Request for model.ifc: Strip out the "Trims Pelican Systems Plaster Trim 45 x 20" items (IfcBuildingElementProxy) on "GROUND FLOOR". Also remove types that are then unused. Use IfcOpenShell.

First a look at what the model holds.

```python
import ifcopenshell
import ifcopenshell.util.element

model = ifcopenshell.open("model.ifc")
print(model.schema)
storey = next(s for s in model.by_type("IfcBuildingStorey") if s.Name == "GROUND FLOOR")
proxies = [e for e in ifcopenshell.util.element.get_decomposition(storey) if e.is_a("IfcBuildingElementProxy")]
seen = {}
for e in proxies:
    element_type = ifcopenshell.util.element.get_type(e)
    name = element_type.Name if element_type not in (None, e) else None
    seen[name] = seen.get(name, 0) + 1
for name, count in sorted(seen.items(), key=str):
    print(count, "x", name)
```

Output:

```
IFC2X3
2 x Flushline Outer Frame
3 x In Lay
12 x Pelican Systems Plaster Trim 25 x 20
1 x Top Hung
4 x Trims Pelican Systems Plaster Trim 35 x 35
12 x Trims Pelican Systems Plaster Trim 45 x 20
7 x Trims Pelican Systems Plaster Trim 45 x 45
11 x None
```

```python
import ifcopenshell
import ifcopenshell.api.root
import ifcopenshell.util.element

model = ifcopenshell.open("model.ifc")

storey = next(s for s in model.by_type("IfcBuildingStorey") if s.Name == "GROUND FLOOR")
proxies = [e for e in ifcopenshell.util.element.get_decomposition(storey) if e.is_a("IfcBuildingElementProxy")]
targets = [e for e in proxies if (t := ifcopenshell.util.element.get_type(e)) not in (None, e) and t.Name == "Trims Pelican Systems Plaster Trim 45 x 20"]
types = {ifcopenshell.util.element.get_type(e) for e in targets} - {None, *targets}

for e in targets:
    ifcopenshell.api.root.remove_product(model, product=e)
print(len(targets), "removed")

unused = [t for t in types if not ifcopenshell.util.element.get_types(t)]
for t in unused:
    ifcopenshell.api.root.remove_product(model, product=t)
print(len(unused), "unused types removed")

model.write("model_updated.ifc")
```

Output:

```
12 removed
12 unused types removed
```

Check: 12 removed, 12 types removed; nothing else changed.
